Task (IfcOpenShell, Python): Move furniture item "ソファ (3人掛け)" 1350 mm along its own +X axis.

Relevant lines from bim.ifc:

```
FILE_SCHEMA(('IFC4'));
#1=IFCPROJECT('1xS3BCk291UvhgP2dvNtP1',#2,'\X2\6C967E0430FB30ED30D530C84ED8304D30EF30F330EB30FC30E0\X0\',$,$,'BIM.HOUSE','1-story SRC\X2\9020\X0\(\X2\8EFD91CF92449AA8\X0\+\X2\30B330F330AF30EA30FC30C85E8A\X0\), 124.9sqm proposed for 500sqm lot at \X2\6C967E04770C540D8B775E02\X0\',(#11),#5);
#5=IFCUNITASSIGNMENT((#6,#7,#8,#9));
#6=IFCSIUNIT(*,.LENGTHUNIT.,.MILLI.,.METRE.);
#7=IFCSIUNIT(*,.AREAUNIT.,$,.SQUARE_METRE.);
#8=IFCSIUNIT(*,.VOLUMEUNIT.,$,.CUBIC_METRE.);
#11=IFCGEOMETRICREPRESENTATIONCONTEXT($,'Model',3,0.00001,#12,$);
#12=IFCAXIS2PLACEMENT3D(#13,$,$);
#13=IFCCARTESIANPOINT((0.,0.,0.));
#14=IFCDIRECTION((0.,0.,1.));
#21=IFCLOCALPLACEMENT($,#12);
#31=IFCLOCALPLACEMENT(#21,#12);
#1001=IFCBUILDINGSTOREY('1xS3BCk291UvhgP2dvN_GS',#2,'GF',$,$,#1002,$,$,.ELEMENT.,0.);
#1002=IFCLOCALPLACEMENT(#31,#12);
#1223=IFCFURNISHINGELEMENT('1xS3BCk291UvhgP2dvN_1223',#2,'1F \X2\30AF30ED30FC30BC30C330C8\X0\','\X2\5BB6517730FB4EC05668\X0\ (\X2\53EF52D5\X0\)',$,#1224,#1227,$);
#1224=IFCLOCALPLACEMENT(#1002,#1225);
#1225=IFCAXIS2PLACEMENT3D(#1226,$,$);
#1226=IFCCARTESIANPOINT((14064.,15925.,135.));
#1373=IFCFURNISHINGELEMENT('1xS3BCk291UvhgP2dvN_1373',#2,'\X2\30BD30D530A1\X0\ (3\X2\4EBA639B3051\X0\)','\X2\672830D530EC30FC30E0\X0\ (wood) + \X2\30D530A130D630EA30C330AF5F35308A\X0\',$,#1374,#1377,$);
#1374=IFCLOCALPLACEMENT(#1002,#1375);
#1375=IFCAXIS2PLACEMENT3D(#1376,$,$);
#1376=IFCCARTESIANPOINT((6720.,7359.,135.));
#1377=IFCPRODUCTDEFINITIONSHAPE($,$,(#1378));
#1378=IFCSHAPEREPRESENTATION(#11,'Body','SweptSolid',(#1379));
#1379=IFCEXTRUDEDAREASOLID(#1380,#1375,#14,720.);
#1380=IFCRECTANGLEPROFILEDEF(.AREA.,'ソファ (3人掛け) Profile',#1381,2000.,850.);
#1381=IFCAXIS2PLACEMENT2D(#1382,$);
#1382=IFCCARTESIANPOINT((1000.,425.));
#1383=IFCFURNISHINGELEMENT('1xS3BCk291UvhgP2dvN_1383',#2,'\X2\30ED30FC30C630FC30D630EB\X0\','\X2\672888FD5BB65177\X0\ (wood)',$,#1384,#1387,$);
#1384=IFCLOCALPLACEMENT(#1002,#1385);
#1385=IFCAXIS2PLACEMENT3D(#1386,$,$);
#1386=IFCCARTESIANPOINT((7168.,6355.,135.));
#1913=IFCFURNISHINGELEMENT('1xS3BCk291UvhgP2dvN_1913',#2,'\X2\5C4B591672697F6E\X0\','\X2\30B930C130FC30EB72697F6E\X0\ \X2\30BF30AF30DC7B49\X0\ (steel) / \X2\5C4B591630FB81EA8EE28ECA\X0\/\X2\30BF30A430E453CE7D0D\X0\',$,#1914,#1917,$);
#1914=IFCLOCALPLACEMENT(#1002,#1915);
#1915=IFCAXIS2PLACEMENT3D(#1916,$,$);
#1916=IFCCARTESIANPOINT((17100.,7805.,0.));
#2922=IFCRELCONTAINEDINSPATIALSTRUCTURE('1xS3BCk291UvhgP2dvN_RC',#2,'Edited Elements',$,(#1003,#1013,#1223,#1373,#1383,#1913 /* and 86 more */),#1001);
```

```python
import ifcopenshell
import ifcopenshell.api.geometry
import ifcopenshell.util.placement
import ifcopenshell.util.unit

model = ifcopenshell.open("bim.ifc")
unit_scale = ifcopenshell.util.unit.calculate_unit_scale(model)

item = model.by_guid("1xS3BCk291UvhgP2dvN_1373")
matrix = ifcopenshell.util.placement.get_local_placement(item.ObjectPlacement)
matrix[:3, 3] += matrix[:3, 0] * 1.35 / unit_scale
ifcopenshell.api.geometry.edit_object_placement(model, product=item, matrix=matrix, is_si=False)

print(ifcopenshell.util.placement.get_local_placement(item.ObjectPlacement).round(3) + 0.0)

model.write("bim_updated.ifc")
```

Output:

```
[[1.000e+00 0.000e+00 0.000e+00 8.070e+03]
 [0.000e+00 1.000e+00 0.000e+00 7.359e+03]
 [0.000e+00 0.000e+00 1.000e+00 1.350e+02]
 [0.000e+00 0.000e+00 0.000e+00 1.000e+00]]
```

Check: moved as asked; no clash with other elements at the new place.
